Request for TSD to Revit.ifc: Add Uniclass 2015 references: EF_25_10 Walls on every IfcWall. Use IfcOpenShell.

First a look at what the model holds.

```python
import ifcopenshell

model = ifcopenshell.open("TSD to Revit.ifc")
print(model.schema)
print("classifications:", [c.Name for c in model.by_type("IfcClassification")])
for ifc_class in ("IfcDoor", "IfcRoof", "IfcStair", "IfcWall", "IfcWindow"):
    print(ifc_class, len(model.by_type(ifc_class)))
```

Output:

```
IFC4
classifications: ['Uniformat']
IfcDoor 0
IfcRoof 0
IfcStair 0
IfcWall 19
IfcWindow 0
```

```python
import ifcopenshell
import ifcopenshell.api.classification

model = ifcopenshell.open("TSD to Revit.ifc")

system = ifcopenshell.api.classification.add_classification(model, classification="Uniclass 2015")

codes = {
    "IfcWall": ("EF_25_10", "Walls"),
}
for ifc_class, (code, name) in codes.items():
    products = model.by_type(ifc_class)
    ifcopenshell.api.classification.add_reference(
        model, products=products, classification=system, identification=code, name=name
    )
    print(code, len(products))

model.write("TSD to Revit_updated.ifc")
```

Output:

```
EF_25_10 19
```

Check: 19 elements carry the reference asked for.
